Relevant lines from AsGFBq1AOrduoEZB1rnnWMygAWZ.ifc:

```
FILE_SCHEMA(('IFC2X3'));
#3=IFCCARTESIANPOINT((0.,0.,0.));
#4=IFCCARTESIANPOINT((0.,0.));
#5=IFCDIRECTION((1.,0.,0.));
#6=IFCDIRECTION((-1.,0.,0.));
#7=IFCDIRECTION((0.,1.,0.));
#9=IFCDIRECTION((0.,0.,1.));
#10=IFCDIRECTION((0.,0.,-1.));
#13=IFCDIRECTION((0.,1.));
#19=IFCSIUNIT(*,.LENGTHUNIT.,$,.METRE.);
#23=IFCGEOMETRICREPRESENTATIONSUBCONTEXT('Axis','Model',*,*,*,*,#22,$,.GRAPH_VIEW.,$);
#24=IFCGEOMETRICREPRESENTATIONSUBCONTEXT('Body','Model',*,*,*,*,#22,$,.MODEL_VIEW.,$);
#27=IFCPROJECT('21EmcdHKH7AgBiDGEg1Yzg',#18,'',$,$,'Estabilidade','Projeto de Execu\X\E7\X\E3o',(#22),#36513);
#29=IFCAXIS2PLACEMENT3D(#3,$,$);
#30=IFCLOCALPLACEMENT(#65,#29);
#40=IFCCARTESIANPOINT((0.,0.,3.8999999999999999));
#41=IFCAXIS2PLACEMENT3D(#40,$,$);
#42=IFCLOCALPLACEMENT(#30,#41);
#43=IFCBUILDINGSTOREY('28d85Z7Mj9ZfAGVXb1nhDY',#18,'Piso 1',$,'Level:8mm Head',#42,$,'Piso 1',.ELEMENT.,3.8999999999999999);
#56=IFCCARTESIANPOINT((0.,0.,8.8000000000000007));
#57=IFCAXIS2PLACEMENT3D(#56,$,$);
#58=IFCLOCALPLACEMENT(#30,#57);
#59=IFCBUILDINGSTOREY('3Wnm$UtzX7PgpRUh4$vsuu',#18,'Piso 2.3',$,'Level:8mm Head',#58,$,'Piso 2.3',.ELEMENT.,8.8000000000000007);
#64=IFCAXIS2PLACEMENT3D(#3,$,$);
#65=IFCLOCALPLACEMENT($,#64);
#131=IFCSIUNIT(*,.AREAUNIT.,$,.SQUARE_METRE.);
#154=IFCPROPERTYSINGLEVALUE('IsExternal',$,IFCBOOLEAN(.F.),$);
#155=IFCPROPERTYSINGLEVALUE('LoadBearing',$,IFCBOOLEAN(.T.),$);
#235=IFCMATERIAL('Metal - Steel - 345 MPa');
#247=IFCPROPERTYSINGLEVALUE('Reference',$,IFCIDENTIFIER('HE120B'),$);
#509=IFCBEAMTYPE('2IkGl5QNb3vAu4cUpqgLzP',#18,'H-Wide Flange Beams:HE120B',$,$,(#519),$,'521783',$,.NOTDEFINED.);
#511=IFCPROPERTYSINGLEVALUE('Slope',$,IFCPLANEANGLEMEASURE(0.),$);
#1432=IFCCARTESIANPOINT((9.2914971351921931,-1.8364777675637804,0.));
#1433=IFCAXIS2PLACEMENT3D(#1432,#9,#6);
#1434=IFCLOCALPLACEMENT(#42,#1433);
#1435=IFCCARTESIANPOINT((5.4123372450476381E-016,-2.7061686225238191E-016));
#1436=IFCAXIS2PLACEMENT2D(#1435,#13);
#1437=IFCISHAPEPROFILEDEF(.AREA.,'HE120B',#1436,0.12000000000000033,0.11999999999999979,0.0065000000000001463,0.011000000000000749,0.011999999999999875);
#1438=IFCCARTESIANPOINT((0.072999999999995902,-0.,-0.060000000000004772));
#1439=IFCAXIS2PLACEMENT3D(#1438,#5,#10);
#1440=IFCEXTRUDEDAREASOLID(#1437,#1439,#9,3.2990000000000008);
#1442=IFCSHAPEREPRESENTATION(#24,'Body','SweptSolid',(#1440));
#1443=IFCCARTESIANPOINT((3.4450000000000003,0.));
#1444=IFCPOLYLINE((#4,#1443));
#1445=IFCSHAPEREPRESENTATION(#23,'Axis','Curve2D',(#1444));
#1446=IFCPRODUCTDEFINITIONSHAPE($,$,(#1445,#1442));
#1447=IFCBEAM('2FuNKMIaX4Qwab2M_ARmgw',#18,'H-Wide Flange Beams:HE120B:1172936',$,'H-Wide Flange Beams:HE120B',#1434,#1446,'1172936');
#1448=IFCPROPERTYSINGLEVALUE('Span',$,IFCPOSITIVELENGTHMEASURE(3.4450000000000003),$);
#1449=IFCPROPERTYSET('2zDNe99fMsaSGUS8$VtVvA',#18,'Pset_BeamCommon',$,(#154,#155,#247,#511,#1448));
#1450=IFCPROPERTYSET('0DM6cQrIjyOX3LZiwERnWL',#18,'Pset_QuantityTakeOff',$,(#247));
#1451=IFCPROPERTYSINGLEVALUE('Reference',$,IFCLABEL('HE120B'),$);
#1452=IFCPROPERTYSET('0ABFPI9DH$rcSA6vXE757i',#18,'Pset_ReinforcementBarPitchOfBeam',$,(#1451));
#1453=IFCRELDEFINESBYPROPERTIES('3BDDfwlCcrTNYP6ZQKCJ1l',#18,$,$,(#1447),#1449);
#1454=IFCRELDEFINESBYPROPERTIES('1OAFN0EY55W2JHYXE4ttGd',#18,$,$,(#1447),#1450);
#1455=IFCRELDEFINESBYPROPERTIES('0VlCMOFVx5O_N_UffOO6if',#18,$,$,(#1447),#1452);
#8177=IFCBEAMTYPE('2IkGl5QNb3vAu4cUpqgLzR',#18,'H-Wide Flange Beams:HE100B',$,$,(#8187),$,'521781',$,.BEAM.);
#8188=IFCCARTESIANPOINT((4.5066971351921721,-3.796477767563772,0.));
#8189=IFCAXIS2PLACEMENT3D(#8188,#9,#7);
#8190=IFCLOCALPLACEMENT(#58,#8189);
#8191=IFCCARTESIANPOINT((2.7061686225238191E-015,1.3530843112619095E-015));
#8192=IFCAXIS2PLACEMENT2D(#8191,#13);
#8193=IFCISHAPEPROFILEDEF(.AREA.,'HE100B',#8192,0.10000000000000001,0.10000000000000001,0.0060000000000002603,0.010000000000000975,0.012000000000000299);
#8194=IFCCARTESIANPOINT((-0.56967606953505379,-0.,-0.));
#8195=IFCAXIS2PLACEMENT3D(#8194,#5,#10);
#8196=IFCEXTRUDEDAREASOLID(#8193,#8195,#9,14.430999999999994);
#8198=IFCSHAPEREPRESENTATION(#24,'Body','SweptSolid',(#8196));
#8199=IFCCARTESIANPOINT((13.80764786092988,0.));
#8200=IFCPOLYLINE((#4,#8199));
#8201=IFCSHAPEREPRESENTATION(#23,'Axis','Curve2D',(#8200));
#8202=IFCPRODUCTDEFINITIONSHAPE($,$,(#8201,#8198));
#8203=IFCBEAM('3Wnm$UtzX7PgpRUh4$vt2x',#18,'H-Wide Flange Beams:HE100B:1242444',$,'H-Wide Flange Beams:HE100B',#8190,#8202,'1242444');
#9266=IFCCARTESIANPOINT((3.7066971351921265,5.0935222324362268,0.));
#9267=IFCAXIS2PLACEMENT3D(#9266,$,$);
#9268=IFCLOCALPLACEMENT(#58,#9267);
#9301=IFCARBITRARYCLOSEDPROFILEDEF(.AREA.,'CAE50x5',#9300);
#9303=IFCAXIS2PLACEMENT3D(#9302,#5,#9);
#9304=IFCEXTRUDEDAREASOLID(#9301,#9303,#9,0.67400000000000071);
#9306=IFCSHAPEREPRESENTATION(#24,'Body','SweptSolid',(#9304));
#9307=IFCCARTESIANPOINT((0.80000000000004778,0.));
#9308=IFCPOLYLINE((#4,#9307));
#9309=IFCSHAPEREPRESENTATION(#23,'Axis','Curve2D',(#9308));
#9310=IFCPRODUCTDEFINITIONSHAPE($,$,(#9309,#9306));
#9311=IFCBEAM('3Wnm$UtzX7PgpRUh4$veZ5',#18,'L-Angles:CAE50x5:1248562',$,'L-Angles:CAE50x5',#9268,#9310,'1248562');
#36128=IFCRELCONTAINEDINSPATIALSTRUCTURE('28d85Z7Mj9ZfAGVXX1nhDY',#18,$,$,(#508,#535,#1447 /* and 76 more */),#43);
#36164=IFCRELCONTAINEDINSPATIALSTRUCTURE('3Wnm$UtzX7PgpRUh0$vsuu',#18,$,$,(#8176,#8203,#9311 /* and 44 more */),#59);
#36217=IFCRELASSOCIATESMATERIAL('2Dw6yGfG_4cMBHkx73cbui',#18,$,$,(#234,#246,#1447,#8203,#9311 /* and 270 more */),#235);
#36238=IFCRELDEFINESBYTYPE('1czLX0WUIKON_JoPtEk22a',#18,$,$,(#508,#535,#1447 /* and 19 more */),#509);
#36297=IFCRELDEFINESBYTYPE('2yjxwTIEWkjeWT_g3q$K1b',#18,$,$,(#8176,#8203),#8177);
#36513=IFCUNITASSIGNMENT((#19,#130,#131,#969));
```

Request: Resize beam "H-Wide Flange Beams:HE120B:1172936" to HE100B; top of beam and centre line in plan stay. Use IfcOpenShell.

```python
import ifcopenshell
import ifcopenshell.api.pset
import ifcopenshell.api.type
import ifcopenshell.util.element
import ifcopenshell.util.representation

model = ifcopenshell.open("AsGFBq1AOrduoEZB1rnnWMygAWZ.ifc")

member = model.by_id(1447)
source = next(p for p in model.by_type("IfcIShapeProfileDef") if p.ProfileName == "HE100B")

body = ifcopenshell.util.representation.get_representation(member, "Model", "Body")
solid = body.Items[0]
old_profile = solid.SweptArea

# Copy the section's sizes but keep this member's own profile position.
profile = ifcopenshell.util.element.copy(model, source)
# Profiles are centred, so shift by half the change in depth to hold the top.
shift = (old_profile.OverallDepth - profile.OverallDepth) / 2
x, y = old_profile.Position.Location.Coordinates
up = (-1.0, 0.0)  # upwards, in the solid's own plane
location = model.createIfcCartesianPoint((x + up[0] * shift, y + up[1] * shift))
profile.Position = model.createIfcAxis2Placement2D(location, old_profile.Position.RefDirection)
solid.SweptArea = profile
if not model.get_total_inverses(old_profile):
    ifcopenshell.util.element.remove_deep2(model, old_profile)

new_type = model.by_guid("2IkGl5QNb3vAu4cUpqgLzR")
ifcopenshell.api.type.assign_type(
    model, related_objects=[member], relating_type=new_type, should_map_representations=False
)
member.Name = member.Name.replace("HE120B", "HE100B")
member.ObjectType = "H-Wide Flange Beams:HE100B"
pset = model.by_id(ifcopenshell.util.element.get_pset(member, "Pset_BeamCommon", should_inherit=False)["id"])
ifcopenshell.api.pset.edit_pset(model, pset=pset, properties={"Reference": "HE100B"})
pset = model.by_id(ifcopenshell.util.element.get_pset(member, "Pset_QuantityTakeOff", should_inherit=False)["id"])
ifcopenshell.api.pset.edit_pset(model, pset=pset, properties={"Reference": "HE100B"})
pset = model.by_id(ifcopenshell.util.element.get_pset(member, "Pset_ReinforcementBarPitchOfBeam", should_inherit=False)["id"])
ifcopenshell.api.pset.edit_pset(model, pset=pset, properties={"Reference": "HE100B"})

print(solid.SweptArea)

model.write("AsGFBq1AOrduoEZB1rnnWMygAWZ_edited.ifc")
```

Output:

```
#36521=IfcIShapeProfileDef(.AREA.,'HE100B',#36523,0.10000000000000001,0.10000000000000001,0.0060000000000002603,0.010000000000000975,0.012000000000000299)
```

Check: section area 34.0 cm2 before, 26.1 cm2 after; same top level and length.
